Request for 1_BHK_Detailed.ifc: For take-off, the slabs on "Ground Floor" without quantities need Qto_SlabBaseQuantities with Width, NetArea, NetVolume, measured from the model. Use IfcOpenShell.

First a look at what the model holds.

```python
import ifcopenshell
import ifcopenshell.util.element
import ifcopenshell.util.unit

model = ifcopenshell.open("1_BHK_Detailed.ifc")
print(model.schema)
for unit_type in ("LENGTHUNIT", "AREAUNIT", "VOLUMEUNIT"):
    print(unit_type, ifcopenshell.util.unit.calculate_unit_scale(model, unit_type))
storey = next(s for s in model.by_type("IfcBuildingStorey") if s.Name == "Ground Floor")
slabs = [e for e in ifcopenshell.util.element.get_decomposition(storey) if e.is_a("IfcSlab")]
for e in sorted(slabs, key=lambda e: e.id()):
    print(e.id(), e.is_a(), e.Name, list(ifcopenshell.util.element.get_psets(e, qtos_only=True)), sep=" | ")
```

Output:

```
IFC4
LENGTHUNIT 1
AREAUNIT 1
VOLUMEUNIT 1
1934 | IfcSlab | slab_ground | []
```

```python
import ifcopenshell
import ifcopenshell.api.pset
import ifcopenshell.geom
import ifcopenshell.util.element
import ifcopenshell.util.shape
import ifcopenshell.util.unit

model = ifcopenshell.open("1_BHK_Detailed.ifc")
unit_scale = ifcopenshell.util.unit.calculate_unit_scale(model)
area_scale = ifcopenshell.util.unit.calculate_unit_scale(model, "AREAUNIT")
volume_scale = ifcopenshell.util.unit.calculate_unit_scale(model, "VOLUMEUNIT")
settings = ifcopenshell.geom.settings()

storey = next(s for s in model.by_type("IfcBuildingStorey") if s.Name == "Ground Floor")
slabs = [e for e in ifcopenshell.util.element.get_decomposition(storey) if e.is_a("IfcSlab")]

for e in sorted(slabs, key=lambda e: e.id()):
    if ifcopenshell.util.element.get_psets(e, qtos_only=True, should_inherit=False):
        continue
    # Geometry comes back in metres, in the element's own axes.
    shape = ifcopenshell.geom.create_shape(settings, e)
    values = {
        "Width": ifcopenshell.util.shape.get_z(shape.geometry) / unit_scale,
        "NetArea": ifcopenshell.util.shape.get_footprint_area(shape.geometry) / area_scale,
        "NetVolume": ifcopenshell.util.shape.get_volume(shape.geometry) / volume_scale,
    }
    qto = ifcopenshell.api.pset.add_qto(model, product=e, name="Qto_SlabBaseQuantities")
    ifcopenshell.api.pset.edit_qto(model, qto=qto, properties=values)
    print(e.id(), {k: round(v, 3) for k, v in values.items()})

model.write("1_BHK_Detailed-out.ifc")
```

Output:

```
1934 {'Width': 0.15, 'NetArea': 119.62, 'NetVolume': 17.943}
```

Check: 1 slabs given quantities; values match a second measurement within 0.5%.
